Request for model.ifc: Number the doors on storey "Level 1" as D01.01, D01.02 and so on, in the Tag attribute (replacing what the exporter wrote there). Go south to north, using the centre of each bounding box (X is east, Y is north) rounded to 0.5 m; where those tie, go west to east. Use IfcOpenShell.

First a look at what the model holds.

```python
import ifcopenshell
import ifcopenshell.util.element
import ifcopenshell.util.placement

model = ifcopenshell.open("model.ifc")
print(model.schema)
storey = next(s for s in model.by_type("IfcBuildingStorey") if s.Name == "Level 1")
doors = [e for e in ifcopenshell.util.element.get_decomposition(storey) if e.is_a("IfcDoor")]
for e in sorted(doors, key=lambda e: e.id()):
    origin = ifcopenshell.util.placement.get_local_placement(e.ObjectPlacement)[:3, 3]
    print(e.id(), e.Tag, e.Name, origin.round(2) + 0.0, sep=" | ")
```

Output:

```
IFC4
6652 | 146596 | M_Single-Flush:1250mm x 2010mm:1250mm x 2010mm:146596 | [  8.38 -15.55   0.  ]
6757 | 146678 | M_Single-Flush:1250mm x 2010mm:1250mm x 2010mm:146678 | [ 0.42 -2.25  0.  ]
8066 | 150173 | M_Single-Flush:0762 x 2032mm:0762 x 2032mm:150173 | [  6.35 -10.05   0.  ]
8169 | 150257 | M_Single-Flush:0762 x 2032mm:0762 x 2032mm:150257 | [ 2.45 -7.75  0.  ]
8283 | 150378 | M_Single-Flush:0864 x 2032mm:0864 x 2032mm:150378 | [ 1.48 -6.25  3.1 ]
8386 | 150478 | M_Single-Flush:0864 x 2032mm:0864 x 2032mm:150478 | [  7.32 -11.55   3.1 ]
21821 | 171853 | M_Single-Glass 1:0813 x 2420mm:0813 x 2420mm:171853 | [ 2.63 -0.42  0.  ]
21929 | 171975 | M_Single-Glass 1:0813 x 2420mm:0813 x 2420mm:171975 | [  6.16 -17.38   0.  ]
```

```python
import ifcopenshell
import ifcopenshell.geom
import ifcopenshell.util.element
import ifcopenshell.util.shape

model = ifcopenshell.open("model.ifc")
settings = ifcopenshell.geom.settings()
settings.set("use-world-coords", True)


def centre(element):
    shape = ifcopenshell.geom.create_shape(settings, element)
    return ifcopenshell.util.shape.get_bbox_centroid(shape.geometry)


storey = next(s for s in model.by_type("IfcBuildingStorey") if s.Name == "Level 1")
doors = [e for e in ifcopenshell.util.element.get_decomposition(storey) if e.is_a("IfcDoor")]

# Insertion points can sit at a corner or the storey origin, so sort by the geometry (in metres).
centres = {e: centre(e) for e in doors}
doors.sort(key=lambda e: (round(centres[e][1] / 0.5), centres[e][0]))

for i, e in enumerate(doors, start=1):
    number = f"D01.{i:02d}"
    e.Tag = number
    print(e.id(), number)

model.write("model_rev.ifc")
```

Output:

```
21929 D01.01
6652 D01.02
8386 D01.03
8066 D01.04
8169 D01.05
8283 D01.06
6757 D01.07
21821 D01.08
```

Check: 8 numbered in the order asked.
